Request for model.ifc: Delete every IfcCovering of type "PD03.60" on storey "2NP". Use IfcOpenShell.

First a look at what the model holds.

```python
import ifcopenshell
import ifcopenshell.util.element

model = ifcopenshell.open("model.ifc")
print(model.schema)
storey = next(s for s in model.by_type("IfcBuildingStorey") if s.Name == "2NP")
coverings = [e for e in ifcopenshell.util.element.get_decomposition(storey) if e.is_a("IfcCovering")]
seen = {}
for e in coverings:
    element_type = ifcopenshell.util.element.get_type(e)
    name = element_type.Name if element_type not in (None, e) else None
    seen[name] = seen.get(name, 0) + 1
for name, count in sorted(seen.items(), key=str):
    print(count, "x", name)
```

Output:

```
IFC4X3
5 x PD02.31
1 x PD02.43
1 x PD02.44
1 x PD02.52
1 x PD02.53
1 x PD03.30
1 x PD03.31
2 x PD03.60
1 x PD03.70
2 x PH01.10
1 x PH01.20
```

```python
import ifcopenshell
import ifcopenshell.api.root
import ifcopenshell.util.element

model = ifcopenshell.open("model.ifc")

storey = next(s for s in model.by_type("IfcBuildingStorey") if s.Name == "2NP")
coverings = [e for e in ifcopenshell.util.element.get_decomposition(storey) if e.is_a("IfcCovering")]
targets = [e for e in coverings if (t := ifcopenshell.util.element.get_type(e)) not in (None, e) and t.Name == "PD03.60"]

for e in targets:
    ifcopenshell.api.root.remove_product(model, product=e)
print(len(targets), "removed")

model.write("model_rev.ifc")
```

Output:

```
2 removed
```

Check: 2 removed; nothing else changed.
